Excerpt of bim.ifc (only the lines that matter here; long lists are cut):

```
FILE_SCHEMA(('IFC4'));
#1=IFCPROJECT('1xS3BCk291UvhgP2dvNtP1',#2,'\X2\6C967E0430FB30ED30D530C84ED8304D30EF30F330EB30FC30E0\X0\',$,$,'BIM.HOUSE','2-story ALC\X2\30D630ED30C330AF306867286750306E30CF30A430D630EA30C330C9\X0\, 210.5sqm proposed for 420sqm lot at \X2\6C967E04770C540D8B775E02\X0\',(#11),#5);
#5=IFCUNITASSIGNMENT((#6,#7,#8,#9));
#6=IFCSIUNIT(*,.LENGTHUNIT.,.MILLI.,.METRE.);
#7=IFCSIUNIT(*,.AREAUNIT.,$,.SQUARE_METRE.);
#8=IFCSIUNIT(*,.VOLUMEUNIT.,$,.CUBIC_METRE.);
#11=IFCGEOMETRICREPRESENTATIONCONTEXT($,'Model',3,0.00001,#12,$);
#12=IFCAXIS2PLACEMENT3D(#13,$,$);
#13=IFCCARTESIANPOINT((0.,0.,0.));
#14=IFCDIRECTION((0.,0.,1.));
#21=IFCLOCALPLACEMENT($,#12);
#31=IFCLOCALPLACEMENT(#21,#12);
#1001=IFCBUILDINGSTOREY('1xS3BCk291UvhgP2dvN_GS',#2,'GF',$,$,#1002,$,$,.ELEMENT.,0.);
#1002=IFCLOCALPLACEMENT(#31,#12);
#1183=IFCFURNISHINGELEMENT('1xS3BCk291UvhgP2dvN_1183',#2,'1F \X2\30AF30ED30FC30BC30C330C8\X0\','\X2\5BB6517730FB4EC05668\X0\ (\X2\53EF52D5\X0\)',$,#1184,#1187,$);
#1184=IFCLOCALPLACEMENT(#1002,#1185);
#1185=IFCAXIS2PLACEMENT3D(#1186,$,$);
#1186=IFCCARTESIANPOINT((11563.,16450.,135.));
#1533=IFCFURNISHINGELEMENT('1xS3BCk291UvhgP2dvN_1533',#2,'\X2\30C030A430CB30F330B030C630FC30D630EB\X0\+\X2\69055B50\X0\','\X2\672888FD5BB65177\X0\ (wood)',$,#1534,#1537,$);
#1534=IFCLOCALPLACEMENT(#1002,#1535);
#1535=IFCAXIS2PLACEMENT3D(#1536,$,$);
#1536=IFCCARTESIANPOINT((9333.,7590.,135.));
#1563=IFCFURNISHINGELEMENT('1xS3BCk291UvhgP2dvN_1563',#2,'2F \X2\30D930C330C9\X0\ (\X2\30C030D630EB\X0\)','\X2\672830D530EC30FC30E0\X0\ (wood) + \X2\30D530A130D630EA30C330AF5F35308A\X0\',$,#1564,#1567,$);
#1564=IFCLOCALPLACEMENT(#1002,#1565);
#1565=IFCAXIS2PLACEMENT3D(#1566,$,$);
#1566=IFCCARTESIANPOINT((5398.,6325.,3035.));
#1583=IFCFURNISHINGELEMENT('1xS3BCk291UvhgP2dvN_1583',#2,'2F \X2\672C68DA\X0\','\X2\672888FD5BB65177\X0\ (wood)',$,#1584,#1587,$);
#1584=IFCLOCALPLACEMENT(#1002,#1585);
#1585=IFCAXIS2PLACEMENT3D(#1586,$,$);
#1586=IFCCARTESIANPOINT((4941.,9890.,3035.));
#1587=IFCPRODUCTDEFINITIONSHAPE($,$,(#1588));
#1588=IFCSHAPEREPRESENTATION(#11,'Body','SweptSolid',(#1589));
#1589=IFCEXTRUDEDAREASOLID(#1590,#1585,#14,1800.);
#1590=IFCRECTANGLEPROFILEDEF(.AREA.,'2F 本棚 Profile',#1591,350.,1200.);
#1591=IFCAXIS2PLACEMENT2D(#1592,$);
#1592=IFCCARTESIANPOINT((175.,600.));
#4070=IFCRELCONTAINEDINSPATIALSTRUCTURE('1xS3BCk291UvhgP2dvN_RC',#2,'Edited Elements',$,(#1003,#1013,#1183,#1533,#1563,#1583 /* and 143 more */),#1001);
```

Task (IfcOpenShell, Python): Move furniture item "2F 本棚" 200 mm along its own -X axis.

```python
import ifcopenshell
import ifcopenshell.api.geometry
import ifcopenshell.util.placement

model = ifcopenshell.open("bim.ifc")

item = model.by_guid("1xS3BCk291UvhgP2dvN_1583")
matrix = ifcopenshell.util.placement.get_local_placement(item.ObjectPlacement)
matrix[:3, 3] -= matrix[:3, 0] * 200.0
ifcopenshell.api.geometry.edit_object_placement(model, product=item, matrix=matrix, is_si=False)

print(ifcopenshell.util.placement.get_local_placement(item.ObjectPlacement).round(3) + 0.0)

model.write("bim_rev.ifc")
```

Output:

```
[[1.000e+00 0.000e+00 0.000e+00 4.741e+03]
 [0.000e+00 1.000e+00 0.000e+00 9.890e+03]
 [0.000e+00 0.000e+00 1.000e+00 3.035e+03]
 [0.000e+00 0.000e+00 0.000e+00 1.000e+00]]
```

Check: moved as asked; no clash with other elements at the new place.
